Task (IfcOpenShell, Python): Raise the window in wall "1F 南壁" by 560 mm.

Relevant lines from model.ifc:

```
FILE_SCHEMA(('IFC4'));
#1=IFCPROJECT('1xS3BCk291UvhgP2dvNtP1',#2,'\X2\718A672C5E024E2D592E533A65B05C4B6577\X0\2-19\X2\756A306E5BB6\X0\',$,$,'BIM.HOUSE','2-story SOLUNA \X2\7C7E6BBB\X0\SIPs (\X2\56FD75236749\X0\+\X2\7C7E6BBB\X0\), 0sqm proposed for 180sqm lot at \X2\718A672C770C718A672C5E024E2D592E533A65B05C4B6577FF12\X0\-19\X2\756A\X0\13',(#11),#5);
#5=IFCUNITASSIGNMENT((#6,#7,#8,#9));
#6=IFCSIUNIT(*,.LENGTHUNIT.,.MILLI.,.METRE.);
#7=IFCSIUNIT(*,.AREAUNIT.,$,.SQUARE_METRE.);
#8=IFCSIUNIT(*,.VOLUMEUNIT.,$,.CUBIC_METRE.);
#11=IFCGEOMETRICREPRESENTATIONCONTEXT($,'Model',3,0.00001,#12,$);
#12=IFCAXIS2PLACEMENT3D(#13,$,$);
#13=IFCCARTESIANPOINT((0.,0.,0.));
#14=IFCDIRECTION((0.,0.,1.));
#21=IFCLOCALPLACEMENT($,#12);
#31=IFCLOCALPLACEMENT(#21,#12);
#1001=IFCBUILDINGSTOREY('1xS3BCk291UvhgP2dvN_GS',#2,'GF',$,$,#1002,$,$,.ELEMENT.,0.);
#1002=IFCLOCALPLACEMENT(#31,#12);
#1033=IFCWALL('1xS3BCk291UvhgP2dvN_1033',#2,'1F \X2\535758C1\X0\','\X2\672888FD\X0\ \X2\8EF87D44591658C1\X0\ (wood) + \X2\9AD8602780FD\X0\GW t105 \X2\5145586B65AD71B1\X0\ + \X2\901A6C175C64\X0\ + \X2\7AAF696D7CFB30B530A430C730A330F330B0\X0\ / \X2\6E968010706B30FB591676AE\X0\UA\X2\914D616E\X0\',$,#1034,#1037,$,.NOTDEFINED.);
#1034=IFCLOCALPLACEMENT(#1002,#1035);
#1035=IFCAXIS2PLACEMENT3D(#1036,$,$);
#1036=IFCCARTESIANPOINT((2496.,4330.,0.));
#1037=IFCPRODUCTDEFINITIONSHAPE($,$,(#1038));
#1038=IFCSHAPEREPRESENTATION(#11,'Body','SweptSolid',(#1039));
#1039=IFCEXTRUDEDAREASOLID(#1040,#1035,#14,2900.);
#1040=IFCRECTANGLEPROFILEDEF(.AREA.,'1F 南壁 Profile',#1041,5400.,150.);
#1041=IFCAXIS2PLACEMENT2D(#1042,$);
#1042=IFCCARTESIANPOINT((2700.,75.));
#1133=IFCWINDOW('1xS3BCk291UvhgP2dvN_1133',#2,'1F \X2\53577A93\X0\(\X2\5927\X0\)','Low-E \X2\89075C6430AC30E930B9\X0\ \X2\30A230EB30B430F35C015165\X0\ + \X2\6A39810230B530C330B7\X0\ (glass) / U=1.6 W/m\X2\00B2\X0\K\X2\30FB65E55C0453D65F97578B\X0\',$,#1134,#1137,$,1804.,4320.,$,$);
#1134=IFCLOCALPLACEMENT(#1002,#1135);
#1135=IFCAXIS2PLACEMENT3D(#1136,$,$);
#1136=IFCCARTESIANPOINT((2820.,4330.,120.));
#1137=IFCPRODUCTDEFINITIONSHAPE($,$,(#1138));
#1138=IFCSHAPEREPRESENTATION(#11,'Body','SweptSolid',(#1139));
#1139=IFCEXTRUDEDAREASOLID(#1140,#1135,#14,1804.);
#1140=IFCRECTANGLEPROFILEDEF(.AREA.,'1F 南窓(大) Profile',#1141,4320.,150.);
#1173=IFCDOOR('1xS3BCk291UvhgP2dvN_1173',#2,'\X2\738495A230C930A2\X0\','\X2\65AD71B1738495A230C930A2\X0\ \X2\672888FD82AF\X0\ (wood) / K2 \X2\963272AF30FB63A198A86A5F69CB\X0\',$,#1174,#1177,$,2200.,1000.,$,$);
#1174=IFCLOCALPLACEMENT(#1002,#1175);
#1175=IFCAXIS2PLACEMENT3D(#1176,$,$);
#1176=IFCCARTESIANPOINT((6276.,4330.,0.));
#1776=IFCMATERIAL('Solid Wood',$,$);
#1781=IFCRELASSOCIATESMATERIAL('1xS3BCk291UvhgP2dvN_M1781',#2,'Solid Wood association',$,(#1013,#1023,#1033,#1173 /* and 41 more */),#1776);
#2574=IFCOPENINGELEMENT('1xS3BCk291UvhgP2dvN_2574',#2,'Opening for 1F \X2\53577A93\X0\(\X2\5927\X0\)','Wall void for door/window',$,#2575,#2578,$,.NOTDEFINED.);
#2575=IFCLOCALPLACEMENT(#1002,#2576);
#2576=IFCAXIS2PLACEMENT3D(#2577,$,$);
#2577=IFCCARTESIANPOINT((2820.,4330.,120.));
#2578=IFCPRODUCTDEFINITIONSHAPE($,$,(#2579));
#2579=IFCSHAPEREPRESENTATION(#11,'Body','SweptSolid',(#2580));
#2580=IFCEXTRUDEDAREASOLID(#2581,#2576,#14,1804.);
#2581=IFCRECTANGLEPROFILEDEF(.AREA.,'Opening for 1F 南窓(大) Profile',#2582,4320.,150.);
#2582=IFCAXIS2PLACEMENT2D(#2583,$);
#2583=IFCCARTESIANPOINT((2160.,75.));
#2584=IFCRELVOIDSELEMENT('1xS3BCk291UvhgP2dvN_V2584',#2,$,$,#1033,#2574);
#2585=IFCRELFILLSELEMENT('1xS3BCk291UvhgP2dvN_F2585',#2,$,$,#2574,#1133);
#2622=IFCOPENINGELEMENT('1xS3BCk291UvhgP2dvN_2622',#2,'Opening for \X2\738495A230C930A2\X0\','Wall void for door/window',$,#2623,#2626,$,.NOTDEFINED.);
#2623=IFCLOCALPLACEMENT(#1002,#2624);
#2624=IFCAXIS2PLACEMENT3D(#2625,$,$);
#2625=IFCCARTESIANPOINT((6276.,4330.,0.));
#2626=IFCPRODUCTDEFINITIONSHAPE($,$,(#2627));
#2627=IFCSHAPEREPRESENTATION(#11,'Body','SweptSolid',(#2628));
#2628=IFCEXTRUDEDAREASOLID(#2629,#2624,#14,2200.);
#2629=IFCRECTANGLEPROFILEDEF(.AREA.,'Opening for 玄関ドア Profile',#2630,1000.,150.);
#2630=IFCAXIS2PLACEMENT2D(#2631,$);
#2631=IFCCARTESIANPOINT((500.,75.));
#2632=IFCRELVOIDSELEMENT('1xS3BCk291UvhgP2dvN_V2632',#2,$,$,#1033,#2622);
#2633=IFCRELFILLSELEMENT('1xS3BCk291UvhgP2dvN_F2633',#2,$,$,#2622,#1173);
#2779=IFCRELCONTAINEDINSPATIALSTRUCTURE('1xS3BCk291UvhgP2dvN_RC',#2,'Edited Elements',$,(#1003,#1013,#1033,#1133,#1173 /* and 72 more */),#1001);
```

```python
import numpy as np
import ifcopenshell
import ifcopenshell.api.geometry
import ifcopenshell.util.placement
import ifcopenshell.util.unit

model = ifcopenshell.open("model.ifc")
unit_scale = ifcopenshell.util.unit.calculate_unit_scale(model)

window = model.by_id(1133)
opening = window.FillsVoids[0].RelatingOpeningElement
dz = 0.56 / unit_scale

shift = np.array([0.0, 0.0, dz])
# The window is not placed relative to its opening, so move both.
for product in (opening, window):
    matrix = ifcopenshell.util.placement.get_local_placement(product.ObjectPlacement)
    matrix[:3, 3] += shift
    ifcopenshell.api.geometry.edit_object_placement(model, product=product, matrix=matrix, is_si=False)

print(f"moved by {dz * unit_scale:+.3f} m")

model.write("model_v2.ifc")
```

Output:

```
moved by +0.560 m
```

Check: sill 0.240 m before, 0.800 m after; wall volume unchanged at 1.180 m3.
